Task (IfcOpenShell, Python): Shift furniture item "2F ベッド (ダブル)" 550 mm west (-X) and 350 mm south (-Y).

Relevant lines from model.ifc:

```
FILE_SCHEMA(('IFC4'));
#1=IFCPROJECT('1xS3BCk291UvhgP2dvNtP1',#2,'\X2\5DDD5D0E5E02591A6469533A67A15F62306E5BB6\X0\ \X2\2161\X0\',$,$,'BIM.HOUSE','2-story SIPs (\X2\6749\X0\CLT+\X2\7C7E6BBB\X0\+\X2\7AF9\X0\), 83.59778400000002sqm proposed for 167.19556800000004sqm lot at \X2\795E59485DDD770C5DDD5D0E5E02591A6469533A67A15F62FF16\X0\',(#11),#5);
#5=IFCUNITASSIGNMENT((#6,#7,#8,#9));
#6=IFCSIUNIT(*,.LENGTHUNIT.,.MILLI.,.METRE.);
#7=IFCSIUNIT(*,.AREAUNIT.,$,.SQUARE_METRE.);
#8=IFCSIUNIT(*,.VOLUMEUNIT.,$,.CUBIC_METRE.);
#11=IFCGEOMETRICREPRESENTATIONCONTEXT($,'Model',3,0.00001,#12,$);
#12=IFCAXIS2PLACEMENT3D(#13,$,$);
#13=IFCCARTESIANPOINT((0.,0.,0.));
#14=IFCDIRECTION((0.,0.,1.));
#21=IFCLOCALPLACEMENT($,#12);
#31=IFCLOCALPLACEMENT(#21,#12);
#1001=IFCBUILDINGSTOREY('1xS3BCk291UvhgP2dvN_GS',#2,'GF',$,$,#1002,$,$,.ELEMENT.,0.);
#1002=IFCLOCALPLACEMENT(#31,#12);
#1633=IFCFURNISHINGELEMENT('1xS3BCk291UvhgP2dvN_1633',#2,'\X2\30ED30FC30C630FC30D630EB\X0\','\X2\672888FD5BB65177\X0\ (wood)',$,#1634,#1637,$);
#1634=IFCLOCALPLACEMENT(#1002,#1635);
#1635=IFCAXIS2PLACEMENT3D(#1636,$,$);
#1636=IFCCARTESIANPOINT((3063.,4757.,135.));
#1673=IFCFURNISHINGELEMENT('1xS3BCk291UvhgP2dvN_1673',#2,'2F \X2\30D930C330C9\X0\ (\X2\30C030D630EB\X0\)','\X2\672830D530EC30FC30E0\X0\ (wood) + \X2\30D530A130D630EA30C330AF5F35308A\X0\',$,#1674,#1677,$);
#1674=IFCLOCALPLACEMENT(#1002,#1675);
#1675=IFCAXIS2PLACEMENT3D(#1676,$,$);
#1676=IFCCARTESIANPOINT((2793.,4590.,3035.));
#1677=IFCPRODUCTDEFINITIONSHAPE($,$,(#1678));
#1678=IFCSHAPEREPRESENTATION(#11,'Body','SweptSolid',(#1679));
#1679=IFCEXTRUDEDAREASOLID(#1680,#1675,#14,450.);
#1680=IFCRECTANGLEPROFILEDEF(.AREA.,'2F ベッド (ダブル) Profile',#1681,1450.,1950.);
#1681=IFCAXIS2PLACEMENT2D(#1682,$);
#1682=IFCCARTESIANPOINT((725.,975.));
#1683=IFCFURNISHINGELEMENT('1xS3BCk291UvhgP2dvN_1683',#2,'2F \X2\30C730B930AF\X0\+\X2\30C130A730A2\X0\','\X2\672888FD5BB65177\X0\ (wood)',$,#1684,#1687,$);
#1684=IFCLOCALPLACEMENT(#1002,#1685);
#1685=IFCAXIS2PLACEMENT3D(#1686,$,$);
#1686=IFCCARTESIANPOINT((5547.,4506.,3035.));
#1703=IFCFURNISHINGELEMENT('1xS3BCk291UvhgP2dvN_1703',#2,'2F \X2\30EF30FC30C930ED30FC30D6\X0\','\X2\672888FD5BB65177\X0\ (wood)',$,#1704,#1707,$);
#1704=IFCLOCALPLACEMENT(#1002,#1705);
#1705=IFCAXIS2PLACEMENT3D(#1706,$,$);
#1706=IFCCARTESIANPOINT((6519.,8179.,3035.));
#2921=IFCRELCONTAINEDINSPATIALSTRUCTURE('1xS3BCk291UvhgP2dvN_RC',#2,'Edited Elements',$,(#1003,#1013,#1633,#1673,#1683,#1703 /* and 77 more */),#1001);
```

```python
import ifcopenshell
import ifcopenshell.api.geometry
import ifcopenshell.util.placement

model = ifcopenshell.open("model.ifc")

item = model.by_guid("1xS3BCk291UvhgP2dvN_1673")
matrix = ifcopenshell.util.placement.get_local_placement(item.ObjectPlacement)
matrix[0, 3] -= 550.0
matrix[1, 3] -= 350.0
ifcopenshell.api.geometry.edit_object_placement(model, product=item, matrix=matrix, is_si=False)

print(ifcopenshell.util.placement.get_local_placement(item.ObjectPlacement).round(3) + 0.0)

model.write("model_v2.ifc")
```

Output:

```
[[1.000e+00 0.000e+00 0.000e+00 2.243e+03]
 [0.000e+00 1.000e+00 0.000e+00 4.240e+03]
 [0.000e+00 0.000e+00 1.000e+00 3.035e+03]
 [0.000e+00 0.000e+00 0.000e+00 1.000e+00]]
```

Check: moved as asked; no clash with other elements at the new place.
